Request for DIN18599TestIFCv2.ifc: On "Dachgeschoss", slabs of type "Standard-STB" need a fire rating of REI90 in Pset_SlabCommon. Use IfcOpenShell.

First a look at what the model holds.

```python
import ifcopenshell
import ifcopenshell.util.element

model = ifcopenshell.open("DIN18599TestIFCv2.ifc")
print(model.schema)
storey = next(s for s in model.by_type("IfcBuildingStorey") if s.Name == "Dachgeschoss")
slabs = [e for e in ifcopenshell.util.element.get_decomposition(storey) if e.is_a("IfcSlab")]
seen = {}
for e in slabs:
    element_type = ifcopenshell.util.element.get_type(e)
    key = (element_type.Name if element_type != e and element_type else None, ifcopenshell.util.element.get_pset(e, "Pset_SlabCommon", "FireRating"))
    seen[key] = seen.get(key, 0) + 1
for (name, value), count in sorted(seen.items(), key=str):
    print(count, "x", name, "|", value)
```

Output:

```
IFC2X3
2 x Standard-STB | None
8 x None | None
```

```python
import ifcopenshell
import ifcopenshell.api.pset
import ifcopenshell.util.element

model = ifcopenshell.open("DIN18599TestIFCv2.ifc")

storey = next(s for s in model.by_type("IfcBuildingStorey") if s.Name == "Dachgeschoss")
slabs = [e for e in ifcopenshell.util.element.get_decomposition(storey) if e.is_a("IfcSlab")]

count = 0
for e in slabs:
    element_type = ifcopenshell.util.element.get_type(e)
    if element_type in (None, e) or element_type.Name != "Standard-STB":
        continue
    # add_pset returns the element's existing set when there is one.
    pset = ifcopenshell.api.pset.add_pset(model, product=e, name="Pset_SlabCommon")
    ifcopenshell.api.pset.edit_pset(model, pset=pset, properties={"FireRating": "REI90"})
    count += 1

print(count, "slabs updated")

model.write("DIN18599TestIFCv2_updated.ifc")
```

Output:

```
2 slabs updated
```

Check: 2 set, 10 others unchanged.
